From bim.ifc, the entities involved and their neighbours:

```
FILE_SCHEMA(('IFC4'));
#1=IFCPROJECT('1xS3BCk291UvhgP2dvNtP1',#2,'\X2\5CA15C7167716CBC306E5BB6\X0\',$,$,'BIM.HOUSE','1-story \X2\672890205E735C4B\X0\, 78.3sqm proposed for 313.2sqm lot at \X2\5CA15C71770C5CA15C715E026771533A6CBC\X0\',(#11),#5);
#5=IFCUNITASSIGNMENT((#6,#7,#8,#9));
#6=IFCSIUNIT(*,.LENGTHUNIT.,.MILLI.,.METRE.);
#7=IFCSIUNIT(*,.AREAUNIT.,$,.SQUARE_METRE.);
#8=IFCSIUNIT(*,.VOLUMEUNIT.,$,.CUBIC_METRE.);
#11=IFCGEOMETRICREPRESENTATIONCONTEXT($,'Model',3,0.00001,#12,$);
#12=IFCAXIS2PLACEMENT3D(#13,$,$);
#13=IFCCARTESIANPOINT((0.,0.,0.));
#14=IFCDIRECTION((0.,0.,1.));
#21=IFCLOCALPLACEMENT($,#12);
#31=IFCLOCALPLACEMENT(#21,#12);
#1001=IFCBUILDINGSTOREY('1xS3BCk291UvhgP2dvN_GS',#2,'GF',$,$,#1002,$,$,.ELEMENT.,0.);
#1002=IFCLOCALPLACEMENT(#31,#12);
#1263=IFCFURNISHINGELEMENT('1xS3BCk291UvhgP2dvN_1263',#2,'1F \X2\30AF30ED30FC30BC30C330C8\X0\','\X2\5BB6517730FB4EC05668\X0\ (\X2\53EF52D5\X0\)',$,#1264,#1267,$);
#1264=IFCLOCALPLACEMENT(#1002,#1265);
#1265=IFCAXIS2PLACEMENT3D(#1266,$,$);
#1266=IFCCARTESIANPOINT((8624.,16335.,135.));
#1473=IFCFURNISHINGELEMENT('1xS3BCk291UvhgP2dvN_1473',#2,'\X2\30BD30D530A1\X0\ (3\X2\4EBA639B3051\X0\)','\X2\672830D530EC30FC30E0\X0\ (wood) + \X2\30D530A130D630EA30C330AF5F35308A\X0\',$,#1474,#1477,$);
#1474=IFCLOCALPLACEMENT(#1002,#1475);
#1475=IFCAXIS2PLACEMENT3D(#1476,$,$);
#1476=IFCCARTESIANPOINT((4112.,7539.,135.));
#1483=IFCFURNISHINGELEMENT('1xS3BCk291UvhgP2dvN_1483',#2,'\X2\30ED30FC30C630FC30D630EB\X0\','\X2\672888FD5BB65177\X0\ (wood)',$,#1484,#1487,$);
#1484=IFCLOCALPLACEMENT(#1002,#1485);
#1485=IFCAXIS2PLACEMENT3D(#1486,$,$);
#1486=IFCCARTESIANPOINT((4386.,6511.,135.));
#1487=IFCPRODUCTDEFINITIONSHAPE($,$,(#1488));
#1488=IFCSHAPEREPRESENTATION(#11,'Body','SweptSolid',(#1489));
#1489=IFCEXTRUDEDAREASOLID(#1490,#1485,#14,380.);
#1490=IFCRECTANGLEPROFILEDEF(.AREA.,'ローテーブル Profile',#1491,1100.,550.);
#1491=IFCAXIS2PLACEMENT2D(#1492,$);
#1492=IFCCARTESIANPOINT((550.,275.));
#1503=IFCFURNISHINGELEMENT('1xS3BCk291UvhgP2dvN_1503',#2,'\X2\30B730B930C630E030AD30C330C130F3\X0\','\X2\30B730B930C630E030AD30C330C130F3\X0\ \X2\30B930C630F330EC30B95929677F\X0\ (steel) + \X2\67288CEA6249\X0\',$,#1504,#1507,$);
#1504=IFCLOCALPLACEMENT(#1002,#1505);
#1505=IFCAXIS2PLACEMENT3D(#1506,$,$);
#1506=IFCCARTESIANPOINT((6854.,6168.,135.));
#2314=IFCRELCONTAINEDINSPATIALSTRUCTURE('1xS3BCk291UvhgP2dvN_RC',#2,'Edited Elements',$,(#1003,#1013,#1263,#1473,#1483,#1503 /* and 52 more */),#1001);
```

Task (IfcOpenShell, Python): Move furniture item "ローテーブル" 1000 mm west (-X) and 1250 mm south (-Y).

```python
import ifcopenshell
import ifcopenshell.api.geometry
import ifcopenshell.util.placement
import ifcopenshell.util.unit

model = ifcopenshell.open("bim.ifc")
unit_scale = ifcopenshell.util.unit.calculate_unit_scale(model)

item = model.by_guid("1xS3BCk291UvhgP2dvN_1483")
matrix = ifcopenshell.util.placement.get_local_placement(item.ObjectPlacement)
matrix[0, 3] -= 1 / unit_scale
matrix[1, 3] -= 1.25 / unit_scale
ifcopenshell.api.geometry.edit_object_placement(model, product=item, matrix=matrix, is_si=False)

print(ifcopenshell.util.placement.get_local_placement(item.ObjectPlacement).round(3) + 0.0)

model.write("bim_edited.ifc")
```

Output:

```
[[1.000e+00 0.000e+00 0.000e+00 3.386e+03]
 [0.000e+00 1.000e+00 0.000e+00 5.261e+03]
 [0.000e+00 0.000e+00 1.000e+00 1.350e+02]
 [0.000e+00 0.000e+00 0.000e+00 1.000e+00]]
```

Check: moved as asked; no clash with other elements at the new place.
